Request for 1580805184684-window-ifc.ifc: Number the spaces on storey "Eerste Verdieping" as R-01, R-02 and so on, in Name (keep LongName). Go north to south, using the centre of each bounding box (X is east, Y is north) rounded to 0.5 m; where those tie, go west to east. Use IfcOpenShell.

First a look at what the model holds.

```python
import ifcopenshell
import ifcopenshell.util.element
import ifcopenshell.util.placement

model = ifcopenshell.open("1580805184684-window-ifc.ifc")
print(model.schema)
storey = next(s for s in model.by_type("IfcBuildingStorey") if s.Name == "Eerste Verdieping")
spaces = [e for e in ifcopenshell.util.element.get_decomposition(storey) if e.is_a("IfcSpace")]
for e in sorted(spaces, key=lambda e: e.id()):
    origin = ifcopenshell.util.placement.get_local_placement(e.ObjectPlacement)[:3, 3]
    print(e.id(), e.Name, e.LongName, origin.round(2) + 0.0, sep=" | ")
```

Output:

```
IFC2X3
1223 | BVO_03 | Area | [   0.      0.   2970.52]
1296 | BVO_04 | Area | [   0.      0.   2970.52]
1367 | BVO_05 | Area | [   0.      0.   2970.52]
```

```python
import ifcopenshell
import ifcopenshell.geom
import ifcopenshell.util.element
import ifcopenshell.util.shape

model = ifcopenshell.open("1580805184684-window-ifc.ifc")
settings = ifcopenshell.geom.settings()
settings.set("use-world-coords", True)


def centre(element):
    shape = ifcopenshell.geom.create_shape(settings, element)
    return ifcopenshell.util.shape.get_bbox_centroid(shape.geometry)


storey = next(s for s in model.by_type("IfcBuildingStorey") if s.Name == "Eerste Verdieping")
spaces = [e for e in ifcopenshell.util.element.get_decomposition(storey) if e.is_a("IfcSpace")]

# Insertion points can sit at a corner or the storey origin, so sort by the geometry (in metres).
centres = {e: centre(e) for e in spaces}
spaces.sort(key=lambda e: (-round(centres[e][1] / 0.5), centres[e][0]))

for i, e in enumerate(spaces, start=1):
    number = f"R-{i:02d}"
    e.Name = number
    print(e.id(), number)

model.write("1580805184684-window-ifc_edited.ifc")
```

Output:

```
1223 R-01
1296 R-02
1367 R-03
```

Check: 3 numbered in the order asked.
